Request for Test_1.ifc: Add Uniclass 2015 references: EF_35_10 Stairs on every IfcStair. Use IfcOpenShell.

First a look at what the model holds.

```python
import ifcopenshell

model = ifcopenshell.open("Test_1.ifc")
print(model.schema)
print("classifications:", [c.Name for c in model.by_type("IfcClassification")])
for ifc_class in ("IfcDoor", "IfcRoof", "IfcStair", "IfcWall", "IfcWindow"):
    print(ifc_class, len(model.by_type(ifc_class)))
```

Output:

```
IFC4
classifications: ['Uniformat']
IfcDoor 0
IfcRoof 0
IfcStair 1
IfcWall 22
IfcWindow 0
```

```python
import ifcopenshell
import ifcopenshell.api.classification

model = ifcopenshell.open("Test_1.ifc")

system = ifcopenshell.api.classification.add_classification(model, classification="Uniclass 2015")

codes = {
    "IfcStair": ("EF_35_10", "Stairs"),
}
for ifc_class, (code, name) in codes.items():
    products = model.by_type(ifc_class)
    ifcopenshell.api.classification.add_reference(
        model, products=products, classification=system, identification=code, name=name
    )
    print(code, len(products))

model.write("Test_1_edited.ifc")
```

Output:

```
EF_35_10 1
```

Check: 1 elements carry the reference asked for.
